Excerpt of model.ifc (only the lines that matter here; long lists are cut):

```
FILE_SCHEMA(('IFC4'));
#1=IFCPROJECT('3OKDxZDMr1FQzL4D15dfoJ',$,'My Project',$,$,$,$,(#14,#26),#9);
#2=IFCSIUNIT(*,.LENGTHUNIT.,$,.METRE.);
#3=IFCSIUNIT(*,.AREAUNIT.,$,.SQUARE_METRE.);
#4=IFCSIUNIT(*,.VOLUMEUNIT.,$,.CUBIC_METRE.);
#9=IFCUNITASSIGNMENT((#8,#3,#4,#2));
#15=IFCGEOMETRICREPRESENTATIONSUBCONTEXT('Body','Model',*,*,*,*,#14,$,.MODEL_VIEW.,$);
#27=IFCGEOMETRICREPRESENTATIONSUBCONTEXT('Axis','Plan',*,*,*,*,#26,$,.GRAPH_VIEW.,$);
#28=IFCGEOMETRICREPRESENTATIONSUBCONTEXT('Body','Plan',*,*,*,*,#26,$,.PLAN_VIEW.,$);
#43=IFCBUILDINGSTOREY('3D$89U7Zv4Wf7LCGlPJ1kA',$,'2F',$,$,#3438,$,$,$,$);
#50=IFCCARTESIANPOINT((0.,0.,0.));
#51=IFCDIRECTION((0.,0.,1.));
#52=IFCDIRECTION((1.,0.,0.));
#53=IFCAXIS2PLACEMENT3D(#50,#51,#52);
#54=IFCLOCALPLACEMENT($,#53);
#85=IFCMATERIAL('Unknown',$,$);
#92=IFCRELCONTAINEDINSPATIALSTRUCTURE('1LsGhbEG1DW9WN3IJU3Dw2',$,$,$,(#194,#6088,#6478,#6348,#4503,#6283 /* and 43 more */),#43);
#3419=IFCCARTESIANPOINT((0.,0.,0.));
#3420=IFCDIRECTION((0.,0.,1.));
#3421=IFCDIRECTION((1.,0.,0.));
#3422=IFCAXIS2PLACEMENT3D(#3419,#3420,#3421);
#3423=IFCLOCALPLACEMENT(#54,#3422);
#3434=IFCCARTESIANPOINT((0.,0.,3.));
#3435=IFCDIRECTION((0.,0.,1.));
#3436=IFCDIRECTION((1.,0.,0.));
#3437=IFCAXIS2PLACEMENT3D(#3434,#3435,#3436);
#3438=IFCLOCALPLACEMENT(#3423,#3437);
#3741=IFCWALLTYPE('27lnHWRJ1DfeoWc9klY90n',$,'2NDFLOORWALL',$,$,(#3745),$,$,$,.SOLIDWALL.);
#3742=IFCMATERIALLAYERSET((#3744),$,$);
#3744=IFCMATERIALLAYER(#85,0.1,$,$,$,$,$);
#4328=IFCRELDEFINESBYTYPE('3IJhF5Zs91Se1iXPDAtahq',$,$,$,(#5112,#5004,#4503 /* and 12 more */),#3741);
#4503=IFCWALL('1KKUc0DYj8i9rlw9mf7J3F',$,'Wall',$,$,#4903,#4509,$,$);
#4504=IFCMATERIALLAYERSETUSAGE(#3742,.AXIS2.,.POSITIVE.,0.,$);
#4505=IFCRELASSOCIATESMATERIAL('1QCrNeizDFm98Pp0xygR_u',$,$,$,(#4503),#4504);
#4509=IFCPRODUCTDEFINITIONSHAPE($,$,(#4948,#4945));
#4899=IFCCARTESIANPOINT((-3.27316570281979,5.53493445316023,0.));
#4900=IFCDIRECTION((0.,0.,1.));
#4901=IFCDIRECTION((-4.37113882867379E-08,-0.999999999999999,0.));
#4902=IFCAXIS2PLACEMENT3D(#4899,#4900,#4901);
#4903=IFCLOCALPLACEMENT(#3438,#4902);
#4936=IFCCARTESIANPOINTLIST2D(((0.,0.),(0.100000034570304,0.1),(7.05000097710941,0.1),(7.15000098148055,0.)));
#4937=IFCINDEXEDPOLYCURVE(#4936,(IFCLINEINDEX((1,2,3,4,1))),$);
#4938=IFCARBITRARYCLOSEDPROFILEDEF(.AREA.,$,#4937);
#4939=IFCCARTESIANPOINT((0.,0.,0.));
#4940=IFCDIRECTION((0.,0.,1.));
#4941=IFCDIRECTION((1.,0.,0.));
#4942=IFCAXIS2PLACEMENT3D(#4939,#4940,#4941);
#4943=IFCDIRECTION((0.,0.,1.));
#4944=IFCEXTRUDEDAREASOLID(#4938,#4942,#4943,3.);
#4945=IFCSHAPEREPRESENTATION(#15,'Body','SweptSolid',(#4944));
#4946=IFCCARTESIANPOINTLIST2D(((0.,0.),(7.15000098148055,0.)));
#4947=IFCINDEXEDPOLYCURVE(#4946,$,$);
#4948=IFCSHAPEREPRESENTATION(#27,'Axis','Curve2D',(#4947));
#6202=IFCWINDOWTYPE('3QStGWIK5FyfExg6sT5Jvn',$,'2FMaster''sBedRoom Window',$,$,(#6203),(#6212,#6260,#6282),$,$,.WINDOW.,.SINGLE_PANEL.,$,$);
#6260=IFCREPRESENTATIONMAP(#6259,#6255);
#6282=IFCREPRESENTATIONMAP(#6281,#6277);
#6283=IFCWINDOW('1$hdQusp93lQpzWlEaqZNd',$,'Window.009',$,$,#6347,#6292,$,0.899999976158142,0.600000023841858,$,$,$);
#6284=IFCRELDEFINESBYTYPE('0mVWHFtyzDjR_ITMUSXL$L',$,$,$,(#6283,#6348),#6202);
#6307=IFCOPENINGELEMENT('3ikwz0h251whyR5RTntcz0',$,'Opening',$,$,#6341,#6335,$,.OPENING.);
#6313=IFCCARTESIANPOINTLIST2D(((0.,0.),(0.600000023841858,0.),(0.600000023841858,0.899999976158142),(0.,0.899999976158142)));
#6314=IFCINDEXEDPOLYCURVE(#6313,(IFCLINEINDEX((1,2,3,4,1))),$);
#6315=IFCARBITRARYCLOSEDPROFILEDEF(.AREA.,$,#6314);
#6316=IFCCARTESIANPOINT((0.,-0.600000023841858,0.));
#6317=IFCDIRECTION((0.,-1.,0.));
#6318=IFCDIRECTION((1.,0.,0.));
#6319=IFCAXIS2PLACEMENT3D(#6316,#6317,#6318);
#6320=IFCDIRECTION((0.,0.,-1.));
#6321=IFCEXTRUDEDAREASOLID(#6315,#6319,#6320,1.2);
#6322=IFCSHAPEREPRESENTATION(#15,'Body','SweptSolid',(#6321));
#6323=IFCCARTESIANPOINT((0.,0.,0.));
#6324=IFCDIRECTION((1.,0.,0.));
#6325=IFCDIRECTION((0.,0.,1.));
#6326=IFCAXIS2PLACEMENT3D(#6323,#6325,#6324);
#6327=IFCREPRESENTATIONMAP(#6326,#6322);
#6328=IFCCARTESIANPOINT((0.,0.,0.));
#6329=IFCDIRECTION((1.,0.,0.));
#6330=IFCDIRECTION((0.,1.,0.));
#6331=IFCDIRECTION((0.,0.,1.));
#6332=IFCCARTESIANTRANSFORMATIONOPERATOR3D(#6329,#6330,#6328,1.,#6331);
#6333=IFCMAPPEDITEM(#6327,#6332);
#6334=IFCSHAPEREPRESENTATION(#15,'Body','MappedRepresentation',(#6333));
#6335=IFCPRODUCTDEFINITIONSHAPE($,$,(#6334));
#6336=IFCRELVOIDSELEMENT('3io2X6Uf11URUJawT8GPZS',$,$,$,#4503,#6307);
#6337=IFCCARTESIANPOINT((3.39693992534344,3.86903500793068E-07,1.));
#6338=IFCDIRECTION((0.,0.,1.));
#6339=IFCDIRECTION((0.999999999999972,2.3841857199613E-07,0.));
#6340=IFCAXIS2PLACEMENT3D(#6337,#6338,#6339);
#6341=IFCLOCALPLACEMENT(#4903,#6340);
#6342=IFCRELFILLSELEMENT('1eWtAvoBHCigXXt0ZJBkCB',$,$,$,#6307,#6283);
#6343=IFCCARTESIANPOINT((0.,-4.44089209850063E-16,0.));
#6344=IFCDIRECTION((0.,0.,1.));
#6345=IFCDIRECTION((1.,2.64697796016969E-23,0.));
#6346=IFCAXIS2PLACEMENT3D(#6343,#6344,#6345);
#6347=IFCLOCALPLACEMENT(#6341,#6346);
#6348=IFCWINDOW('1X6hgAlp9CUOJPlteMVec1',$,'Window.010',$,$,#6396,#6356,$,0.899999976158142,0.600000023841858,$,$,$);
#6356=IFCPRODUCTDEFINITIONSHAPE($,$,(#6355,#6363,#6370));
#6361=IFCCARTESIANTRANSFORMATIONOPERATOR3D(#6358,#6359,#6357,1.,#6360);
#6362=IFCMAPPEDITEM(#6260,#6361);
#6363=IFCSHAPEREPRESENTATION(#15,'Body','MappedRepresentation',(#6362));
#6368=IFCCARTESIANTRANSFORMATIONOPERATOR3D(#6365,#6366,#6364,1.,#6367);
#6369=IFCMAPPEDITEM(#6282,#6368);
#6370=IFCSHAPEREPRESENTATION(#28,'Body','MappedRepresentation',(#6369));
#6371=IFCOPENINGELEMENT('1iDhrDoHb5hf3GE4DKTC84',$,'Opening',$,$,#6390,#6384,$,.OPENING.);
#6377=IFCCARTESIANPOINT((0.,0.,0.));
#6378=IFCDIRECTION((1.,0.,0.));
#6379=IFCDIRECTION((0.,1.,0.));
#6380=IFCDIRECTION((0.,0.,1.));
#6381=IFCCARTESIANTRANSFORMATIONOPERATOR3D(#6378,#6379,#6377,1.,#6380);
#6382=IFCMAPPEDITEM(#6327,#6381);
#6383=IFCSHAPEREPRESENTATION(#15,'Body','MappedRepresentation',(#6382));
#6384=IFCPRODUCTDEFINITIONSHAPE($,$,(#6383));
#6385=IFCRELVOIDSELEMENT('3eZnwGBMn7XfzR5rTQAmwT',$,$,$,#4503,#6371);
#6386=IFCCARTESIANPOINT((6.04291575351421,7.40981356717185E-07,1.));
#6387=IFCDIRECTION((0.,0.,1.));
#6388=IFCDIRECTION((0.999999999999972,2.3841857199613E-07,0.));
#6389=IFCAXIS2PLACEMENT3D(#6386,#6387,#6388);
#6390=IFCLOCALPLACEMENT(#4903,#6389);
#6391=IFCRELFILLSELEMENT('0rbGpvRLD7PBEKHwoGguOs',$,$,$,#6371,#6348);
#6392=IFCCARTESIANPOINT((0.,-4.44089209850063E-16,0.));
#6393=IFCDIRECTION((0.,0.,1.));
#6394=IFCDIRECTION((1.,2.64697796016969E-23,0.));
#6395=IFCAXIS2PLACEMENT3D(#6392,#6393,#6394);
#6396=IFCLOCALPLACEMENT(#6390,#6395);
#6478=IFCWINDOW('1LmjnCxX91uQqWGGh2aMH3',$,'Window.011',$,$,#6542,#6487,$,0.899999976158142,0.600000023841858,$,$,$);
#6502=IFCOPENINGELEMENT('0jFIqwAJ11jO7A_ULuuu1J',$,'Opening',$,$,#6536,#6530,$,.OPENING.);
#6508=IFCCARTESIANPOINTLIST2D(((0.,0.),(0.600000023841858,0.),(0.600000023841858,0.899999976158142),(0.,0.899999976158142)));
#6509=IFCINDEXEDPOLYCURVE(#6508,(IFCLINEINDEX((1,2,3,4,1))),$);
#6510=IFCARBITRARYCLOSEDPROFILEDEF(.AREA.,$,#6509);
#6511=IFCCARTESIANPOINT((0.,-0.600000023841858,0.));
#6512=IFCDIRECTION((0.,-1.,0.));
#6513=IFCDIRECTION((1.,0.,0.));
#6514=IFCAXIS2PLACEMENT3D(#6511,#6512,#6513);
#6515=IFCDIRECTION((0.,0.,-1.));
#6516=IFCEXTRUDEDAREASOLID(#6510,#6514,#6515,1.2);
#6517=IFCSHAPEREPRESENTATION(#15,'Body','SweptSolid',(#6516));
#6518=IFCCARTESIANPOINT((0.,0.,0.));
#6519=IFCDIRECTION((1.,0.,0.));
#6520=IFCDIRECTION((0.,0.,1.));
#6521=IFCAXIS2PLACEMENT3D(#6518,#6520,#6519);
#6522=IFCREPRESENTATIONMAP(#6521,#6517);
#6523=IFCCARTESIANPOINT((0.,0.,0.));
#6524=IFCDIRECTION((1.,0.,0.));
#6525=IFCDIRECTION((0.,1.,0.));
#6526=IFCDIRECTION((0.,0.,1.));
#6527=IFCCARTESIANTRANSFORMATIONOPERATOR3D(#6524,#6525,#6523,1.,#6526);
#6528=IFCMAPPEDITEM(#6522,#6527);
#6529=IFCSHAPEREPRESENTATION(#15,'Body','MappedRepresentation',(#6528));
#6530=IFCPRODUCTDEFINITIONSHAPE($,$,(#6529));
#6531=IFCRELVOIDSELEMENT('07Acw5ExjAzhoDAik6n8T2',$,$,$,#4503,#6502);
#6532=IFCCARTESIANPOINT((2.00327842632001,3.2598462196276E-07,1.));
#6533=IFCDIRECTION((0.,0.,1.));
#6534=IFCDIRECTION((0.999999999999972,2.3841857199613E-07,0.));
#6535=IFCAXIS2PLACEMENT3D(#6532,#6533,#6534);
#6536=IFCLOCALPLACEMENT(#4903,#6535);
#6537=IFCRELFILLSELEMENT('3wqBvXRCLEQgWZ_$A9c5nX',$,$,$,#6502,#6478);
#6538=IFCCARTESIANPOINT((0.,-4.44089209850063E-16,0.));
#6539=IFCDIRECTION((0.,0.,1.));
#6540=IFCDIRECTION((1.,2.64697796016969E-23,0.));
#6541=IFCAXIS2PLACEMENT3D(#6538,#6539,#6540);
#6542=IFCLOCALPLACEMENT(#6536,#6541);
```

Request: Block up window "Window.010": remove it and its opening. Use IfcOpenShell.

```python
import ifcopenshell
import ifcopenshell.api.feature
import ifcopenshell.api.root
import ifcopenshell.geom
import ifcopenshell.util.shape

model = ifcopenshell.open("model.ifc")
settings = ifcopenshell.geom.settings()


def volume(element):
    """Net volume in cubic metres, openings subtracted."""
    shape = ifcopenshell.geom.create_shape(settings, element)
    return ifcopenshell.util.shape.get_volume(shape.geometry)


window = model.by_guid("1X6hgAlp9CUOJPlteMVec1")
opening = window.FillsVoids[0].RelatingOpeningElement
wall = opening.VoidsElements[0].RelatingBuildingElement
before = volume(wall)

ifcopenshell.api.root.remove_product(model, product=window)
ifcopenshell.api.feature.remove_feature(model, feature=opening)

after = volume(wall)

print(f"wall volume {before:.3f} -> {after:.3f} m3")

model.write("model-out.ifc")
```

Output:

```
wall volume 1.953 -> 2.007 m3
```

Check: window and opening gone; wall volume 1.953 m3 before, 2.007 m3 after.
